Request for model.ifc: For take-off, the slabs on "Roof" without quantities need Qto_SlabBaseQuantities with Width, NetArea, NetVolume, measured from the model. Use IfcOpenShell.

First a look at what the model holds.

```python
import ifcopenshell
import ifcopenshell.util.element
import ifcopenshell.util.unit

model = ifcopenshell.open("model.ifc")
print(model.schema)
for unit_type in ("LENGTHUNIT", "AREAUNIT", "VOLUMEUNIT"):
    print(unit_type, ifcopenshell.util.unit.calculate_unit_scale(model, unit_type))
storey = next(s for s in model.by_type("IfcBuildingStorey") if s.Name == "Roof")
slabs = [e for e in ifcopenshell.util.element.get_decomposition(storey) if e.is_a("IfcSlab")]
for e in sorted(slabs, key=lambda e: e.id()):
    print(e.id(), e.is_a(), e.Name, list(ifcopenshell.util.element.get_psets(e, qtos_only=True)), sep=" | ")
```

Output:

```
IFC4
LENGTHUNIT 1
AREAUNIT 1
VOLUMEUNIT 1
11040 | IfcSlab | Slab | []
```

```python
import ifcopenshell
import ifcopenshell.api.pset
import ifcopenshell.geom
import ifcopenshell.util.element
import ifcopenshell.util.shape
import ifcopenshell.util.unit

model = ifcopenshell.open("model.ifc")
unit_scale = ifcopenshell.util.unit.calculate_unit_scale(model)
area_scale = ifcopenshell.util.unit.calculate_unit_scale(model, "AREAUNIT")
volume_scale = ifcopenshell.util.unit.calculate_unit_scale(model, "VOLUMEUNIT")
settings = ifcopenshell.geom.settings()

storey = next(s for s in model.by_type("IfcBuildingStorey") if s.Name == "Roof")
slabs = [e for e in ifcopenshell.util.element.get_decomposition(storey) if e.is_a("IfcSlab")]

for e in sorted(slabs, key=lambda e: e.id()):
    if ifcopenshell.util.element.get_psets(e, qtos_only=True, should_inherit=False):
        continue
    # Geometry comes back in metres, in the element's own axes.
    shape = ifcopenshell.geom.create_shape(settings, e)
    values = {
        "Width": ifcopenshell.util.shape.get_z(shape.geometry) / unit_scale,
        "NetArea": ifcopenshell.util.shape.get_footprint_area(shape.geometry) / area_scale,
        "NetVolume": ifcopenshell.util.shape.get_volume(shape.geometry) / volume_scale,
    }
    qto = ifcopenshell.api.pset.add_qto(model, product=e, name="Qto_SlabBaseQuantities")
    ifcopenshell.api.pset.edit_qto(model, qto=qto, properties=values)
    print(e.id(), {k: round(v, 3) for k, v in values.items()})

model.write("model-out.ifc")
```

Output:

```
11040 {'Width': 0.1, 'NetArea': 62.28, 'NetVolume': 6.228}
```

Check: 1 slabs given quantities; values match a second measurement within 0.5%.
